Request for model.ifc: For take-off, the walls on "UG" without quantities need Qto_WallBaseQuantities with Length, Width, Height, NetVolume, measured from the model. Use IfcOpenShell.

First a look at what the model holds.

```python
import ifcopenshell
import ifcopenshell.util.element
import ifcopenshell.util.unit

model = ifcopenshell.open("model.ifc")
print(model.schema)
for unit_type in ("LENGTHUNIT", "AREAUNIT", "VOLUMEUNIT"):
    print(unit_type, ifcopenshell.util.unit.calculate_unit_scale(model, unit_type))
storey = next(s for s in model.by_type("IfcBuildingStorey") if s.Name == "UG")
walls = [e for e in ifcopenshell.util.element.get_decomposition(storey) if e.is_a("IfcWall")]
for e in sorted(walls, key=lambda e: e.id()):
    print(e.id(), e.is_a(), e.Name, list(ifcopenshell.util.element.get_psets(e, qtos_only=True)), sep=" | ")
```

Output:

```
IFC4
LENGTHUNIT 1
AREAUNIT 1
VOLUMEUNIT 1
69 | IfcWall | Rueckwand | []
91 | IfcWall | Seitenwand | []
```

```python
import ifcopenshell
import ifcopenshell.api.pset
import ifcopenshell.geom
import ifcopenshell.util.element
import ifcopenshell.util.shape
import ifcopenshell.util.unit

model = ifcopenshell.open("model.ifc")
unit_scale = ifcopenshell.util.unit.calculate_unit_scale(model)
volume_scale = ifcopenshell.util.unit.calculate_unit_scale(model, "VOLUMEUNIT")
settings = ifcopenshell.geom.settings()

storey = next(s for s in model.by_type("IfcBuildingStorey") if s.Name == "UG")
walls = [e for e in ifcopenshell.util.element.get_decomposition(storey) if e.is_a("IfcWall")]

for e in sorted(walls, key=lambda e: e.id()):
    if ifcopenshell.util.element.get_psets(e, qtos_only=True, should_inherit=False):
        continue
    # Geometry comes back in metres, in the element's own axes.
    shape = ifcopenshell.geom.create_shape(settings, e)
    values = {
        "Length": ifcopenshell.util.shape.get_x(shape.geometry) / unit_scale,
        "Width": ifcopenshell.util.shape.get_y(shape.geometry) / unit_scale,
        "Height": ifcopenshell.util.shape.get_z(shape.geometry) / unit_scale,
        "NetVolume": ifcopenshell.util.shape.get_volume(shape.geometry) / volume_scale,
    }
    qto = ifcopenshell.api.pset.add_qto(model, product=e, name="Qto_WallBaseQuantities")
    ifcopenshell.api.pset.edit_qto(model, qto=qto, properties=values)
    print(e.id(), {k: round(v, 3) for k, v in values.items()})

model.write("model_updated.ifc")
```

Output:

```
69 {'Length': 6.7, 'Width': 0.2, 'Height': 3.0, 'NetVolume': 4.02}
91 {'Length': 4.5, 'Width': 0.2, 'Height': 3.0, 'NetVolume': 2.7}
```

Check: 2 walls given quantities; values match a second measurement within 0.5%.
